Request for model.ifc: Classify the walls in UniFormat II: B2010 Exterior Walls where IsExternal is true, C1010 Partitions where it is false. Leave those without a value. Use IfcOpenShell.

First a look at what the model holds.

```python
import ifcopenshell
import ifcopenshell.util.element

model = ifcopenshell.open("model.ifc")
print(model.schema)
print("classifications:", [c.Name for c in model.by_type("IfcClassification")])
values = [ifcopenshell.util.element.get_pset(e, "Pset_WallCommon", "IsExternal") for e in model.by_type("IfcWall")]
for value in (True, False, None):
    print("IsExternal", value, values.count(value))
```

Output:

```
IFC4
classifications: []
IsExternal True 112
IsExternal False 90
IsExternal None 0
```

```python
import ifcopenshell
import ifcopenshell.api.classification
import ifcopenshell.util.element

model = ifcopenshell.open("model.ifc")

system = ifcopenshell.api.classification.add_classification(model, classification="UniFormat II")

walls = model.by_type("IfcWall")
external = {e: ifcopenshell.util.element.get_pset(e, "Pset_WallCommon", "IsExternal") for e in walls}
for flag, code, name in ((True, "B2010", "Exterior Walls"), (False, "C1010", "Partitions")):
    products = [e for e in walls if external[e] is flag]
    ifcopenshell.api.classification.add_reference(
        model, products=products, classification=system, identification=code, name=name
    )
    print(code, len(products))

model.write("model-out.ifc")
```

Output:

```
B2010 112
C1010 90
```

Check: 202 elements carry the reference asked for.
